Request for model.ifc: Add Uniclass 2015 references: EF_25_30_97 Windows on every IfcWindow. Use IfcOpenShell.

First a look at what the model holds.

```python
import ifcopenshell

model = ifcopenshell.open("model.ifc")
print(model.schema)
print("classifications:", [c.Name for c in model.by_type("IfcClassification")])
for ifc_class in ("IfcDoor", "IfcRoof", "IfcStair", "IfcWall", "IfcWindow"):
    print(ifc_class, len(model.by_type(ifc_class)))
```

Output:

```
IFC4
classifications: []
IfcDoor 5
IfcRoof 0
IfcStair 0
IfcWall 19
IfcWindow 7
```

```python
import ifcopenshell
import ifcopenshell.api.classification

model = ifcopenshell.open("model.ifc")

system = ifcopenshell.api.classification.add_classification(model, classification="Uniclass 2015")

codes = {
    "IfcWindow": ("EF_25_30_97", "Windows"),
}
for ifc_class, (code, name) in codes.items():
    products = model.by_type(ifc_class)
    ifcopenshell.api.classification.add_reference(
        model, products=products, classification=system, identification=code, name=name
    )
    print(code, len(products))

model.write("model-out.ifc")
```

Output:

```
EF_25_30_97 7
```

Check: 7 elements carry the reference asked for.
